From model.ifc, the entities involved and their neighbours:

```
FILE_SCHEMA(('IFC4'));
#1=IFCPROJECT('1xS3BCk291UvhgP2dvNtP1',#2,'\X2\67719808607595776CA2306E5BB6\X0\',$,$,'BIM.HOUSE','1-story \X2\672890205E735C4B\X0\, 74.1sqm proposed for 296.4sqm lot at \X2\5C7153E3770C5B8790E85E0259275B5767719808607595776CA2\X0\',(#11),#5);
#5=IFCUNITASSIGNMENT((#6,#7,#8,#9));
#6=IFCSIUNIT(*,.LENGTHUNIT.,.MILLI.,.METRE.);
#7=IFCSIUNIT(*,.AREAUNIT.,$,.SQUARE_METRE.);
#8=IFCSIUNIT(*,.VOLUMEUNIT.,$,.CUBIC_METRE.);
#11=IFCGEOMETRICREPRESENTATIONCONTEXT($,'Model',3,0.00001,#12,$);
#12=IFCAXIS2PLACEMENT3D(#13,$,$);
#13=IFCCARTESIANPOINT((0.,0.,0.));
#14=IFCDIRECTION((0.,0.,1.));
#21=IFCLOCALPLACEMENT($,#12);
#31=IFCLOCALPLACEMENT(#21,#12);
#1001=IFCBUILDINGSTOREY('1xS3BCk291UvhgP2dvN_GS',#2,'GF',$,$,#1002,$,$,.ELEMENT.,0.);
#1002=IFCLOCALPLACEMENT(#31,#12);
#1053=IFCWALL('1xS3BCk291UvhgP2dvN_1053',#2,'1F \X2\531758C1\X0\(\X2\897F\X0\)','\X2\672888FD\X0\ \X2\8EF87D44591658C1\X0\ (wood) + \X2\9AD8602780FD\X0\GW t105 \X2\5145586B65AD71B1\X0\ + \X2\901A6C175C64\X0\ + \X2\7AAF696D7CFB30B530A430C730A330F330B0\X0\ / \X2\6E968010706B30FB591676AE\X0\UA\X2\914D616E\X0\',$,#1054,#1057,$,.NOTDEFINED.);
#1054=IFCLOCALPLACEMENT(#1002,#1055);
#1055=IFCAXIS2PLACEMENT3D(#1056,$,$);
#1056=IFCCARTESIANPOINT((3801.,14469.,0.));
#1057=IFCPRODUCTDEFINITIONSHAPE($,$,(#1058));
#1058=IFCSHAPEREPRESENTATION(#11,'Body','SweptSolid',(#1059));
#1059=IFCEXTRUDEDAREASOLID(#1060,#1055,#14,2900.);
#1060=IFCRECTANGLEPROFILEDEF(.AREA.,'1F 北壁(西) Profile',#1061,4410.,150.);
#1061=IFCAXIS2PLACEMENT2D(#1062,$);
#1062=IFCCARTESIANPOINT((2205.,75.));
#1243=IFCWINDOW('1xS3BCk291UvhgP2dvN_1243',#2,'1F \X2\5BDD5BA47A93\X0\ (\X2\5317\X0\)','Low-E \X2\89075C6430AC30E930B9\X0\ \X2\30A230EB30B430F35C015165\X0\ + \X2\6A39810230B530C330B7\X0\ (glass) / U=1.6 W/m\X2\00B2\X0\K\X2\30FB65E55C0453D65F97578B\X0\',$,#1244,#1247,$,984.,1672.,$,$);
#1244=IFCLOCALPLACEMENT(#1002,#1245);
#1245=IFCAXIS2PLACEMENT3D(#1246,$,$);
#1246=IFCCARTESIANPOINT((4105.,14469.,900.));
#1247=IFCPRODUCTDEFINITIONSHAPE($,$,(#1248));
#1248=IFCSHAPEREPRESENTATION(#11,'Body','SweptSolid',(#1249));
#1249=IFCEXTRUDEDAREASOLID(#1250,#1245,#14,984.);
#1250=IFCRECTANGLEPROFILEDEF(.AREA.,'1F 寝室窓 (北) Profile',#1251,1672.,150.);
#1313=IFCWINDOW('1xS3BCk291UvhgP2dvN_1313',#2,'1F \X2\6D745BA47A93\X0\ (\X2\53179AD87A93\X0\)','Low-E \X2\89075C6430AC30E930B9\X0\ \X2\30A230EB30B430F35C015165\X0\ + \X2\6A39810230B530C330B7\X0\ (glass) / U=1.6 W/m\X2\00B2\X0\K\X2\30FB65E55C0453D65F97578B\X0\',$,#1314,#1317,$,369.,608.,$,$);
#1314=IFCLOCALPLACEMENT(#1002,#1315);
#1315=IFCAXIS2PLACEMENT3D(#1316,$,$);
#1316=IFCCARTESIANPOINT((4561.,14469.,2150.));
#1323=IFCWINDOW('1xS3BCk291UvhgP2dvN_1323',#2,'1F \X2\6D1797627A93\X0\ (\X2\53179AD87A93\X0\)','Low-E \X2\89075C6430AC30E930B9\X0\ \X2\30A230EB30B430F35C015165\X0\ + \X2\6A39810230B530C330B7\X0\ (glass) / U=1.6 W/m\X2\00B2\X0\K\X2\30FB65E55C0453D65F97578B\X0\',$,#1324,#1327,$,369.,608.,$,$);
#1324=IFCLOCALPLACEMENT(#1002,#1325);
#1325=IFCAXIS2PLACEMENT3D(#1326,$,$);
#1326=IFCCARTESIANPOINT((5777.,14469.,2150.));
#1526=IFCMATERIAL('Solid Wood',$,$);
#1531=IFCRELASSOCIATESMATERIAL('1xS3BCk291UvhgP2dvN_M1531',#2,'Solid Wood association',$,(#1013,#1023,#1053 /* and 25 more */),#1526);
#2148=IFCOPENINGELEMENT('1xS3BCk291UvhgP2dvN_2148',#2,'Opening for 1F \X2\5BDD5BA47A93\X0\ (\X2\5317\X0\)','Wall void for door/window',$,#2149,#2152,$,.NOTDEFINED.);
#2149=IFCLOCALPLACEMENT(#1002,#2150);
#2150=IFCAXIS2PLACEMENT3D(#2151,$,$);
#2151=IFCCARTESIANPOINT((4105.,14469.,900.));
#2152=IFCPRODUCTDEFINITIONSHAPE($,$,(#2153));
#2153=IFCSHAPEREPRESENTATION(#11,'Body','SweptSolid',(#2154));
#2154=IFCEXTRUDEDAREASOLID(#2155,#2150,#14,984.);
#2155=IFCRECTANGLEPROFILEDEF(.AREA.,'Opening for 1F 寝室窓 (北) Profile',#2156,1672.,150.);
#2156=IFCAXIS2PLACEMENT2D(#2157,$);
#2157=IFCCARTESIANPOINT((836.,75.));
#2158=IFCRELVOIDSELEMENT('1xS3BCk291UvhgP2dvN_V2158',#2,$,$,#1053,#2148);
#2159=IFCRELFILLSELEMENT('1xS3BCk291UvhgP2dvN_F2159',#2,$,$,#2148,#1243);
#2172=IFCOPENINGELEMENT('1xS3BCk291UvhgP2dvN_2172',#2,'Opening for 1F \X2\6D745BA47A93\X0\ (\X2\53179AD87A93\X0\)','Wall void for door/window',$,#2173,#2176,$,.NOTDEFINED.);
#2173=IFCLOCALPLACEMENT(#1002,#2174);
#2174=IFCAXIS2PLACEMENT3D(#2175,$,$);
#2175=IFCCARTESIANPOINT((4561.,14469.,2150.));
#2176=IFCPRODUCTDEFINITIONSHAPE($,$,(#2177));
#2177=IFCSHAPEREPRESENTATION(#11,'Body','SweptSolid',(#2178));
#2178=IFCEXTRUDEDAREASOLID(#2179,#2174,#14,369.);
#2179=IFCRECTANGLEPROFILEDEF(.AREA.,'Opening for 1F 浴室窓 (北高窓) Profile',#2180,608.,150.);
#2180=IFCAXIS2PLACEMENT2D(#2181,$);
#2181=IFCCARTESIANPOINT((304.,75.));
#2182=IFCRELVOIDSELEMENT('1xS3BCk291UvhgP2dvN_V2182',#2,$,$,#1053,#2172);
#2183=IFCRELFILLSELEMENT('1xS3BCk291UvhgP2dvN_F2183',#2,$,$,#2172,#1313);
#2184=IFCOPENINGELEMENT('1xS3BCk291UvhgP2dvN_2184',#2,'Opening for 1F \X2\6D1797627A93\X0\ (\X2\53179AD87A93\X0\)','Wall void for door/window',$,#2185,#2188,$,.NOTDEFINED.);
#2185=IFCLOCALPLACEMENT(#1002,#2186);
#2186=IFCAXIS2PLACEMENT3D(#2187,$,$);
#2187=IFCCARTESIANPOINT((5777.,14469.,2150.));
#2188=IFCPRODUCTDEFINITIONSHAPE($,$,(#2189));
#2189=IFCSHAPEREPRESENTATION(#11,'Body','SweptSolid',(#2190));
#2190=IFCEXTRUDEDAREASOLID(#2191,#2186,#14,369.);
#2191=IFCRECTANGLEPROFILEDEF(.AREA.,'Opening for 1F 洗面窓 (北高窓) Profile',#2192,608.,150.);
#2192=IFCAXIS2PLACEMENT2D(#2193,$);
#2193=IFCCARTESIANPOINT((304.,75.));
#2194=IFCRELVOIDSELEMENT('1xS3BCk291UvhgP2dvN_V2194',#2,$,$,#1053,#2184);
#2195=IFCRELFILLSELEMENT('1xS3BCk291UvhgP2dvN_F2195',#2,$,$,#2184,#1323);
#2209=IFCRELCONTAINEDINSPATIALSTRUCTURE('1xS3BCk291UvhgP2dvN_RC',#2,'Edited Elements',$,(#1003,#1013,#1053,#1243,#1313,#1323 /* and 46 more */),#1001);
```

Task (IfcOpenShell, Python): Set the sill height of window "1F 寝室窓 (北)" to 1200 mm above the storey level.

```python
import numpy as np
import ifcopenshell
import ifcopenshell.api.geometry
import ifcopenshell.geom
import ifcopenshell.util.element
import ifcopenshell.util.placement
import ifcopenshell.util.shape
import ifcopenshell.util.unit

model = ifcopenshell.open("model.ifc")
unit_scale = ifcopenshell.util.unit.calculate_unit_scale(model)

window = model.by_guid("1xS3BCk291UvhgP2dvN_1243")
opening = window.FillsVoids[0].RelatingOpeningElement
storey = ifcopenshell.util.element.get_container(window, ifc_class="IfcBuildingStorey")
level = ifcopenshell.util.placement.get_local_placement(storey.ObjectPlacement)[2, 3]

# The opening's origin need not be at the sill, so measure its lowest point.
shape = ifcopenshell.geom.create_shape(ifcopenshell.geom.settings(), opening)
bottom = ifcopenshell.util.shape.get_shape_bottom_elevation(shape, shape.geometry) / unit_scale
dz = level + 1200.0 - bottom

shift = np.array([0.0, 0.0, dz])
# The window is not placed relative to its opening, so move both.
for product in (opening, window):
    matrix = ifcopenshell.util.placement.get_local_placement(product.ObjectPlacement)
    matrix[:3, 3] += shift
    ifcopenshell.api.geometry.edit_object_placement(model, product=product, matrix=matrix, is_si=False)

print(f"moved by {dz * unit_scale:+.3f} m")

model.write("model_rev.ifc")
```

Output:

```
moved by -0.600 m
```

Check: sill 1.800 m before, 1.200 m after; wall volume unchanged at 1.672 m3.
